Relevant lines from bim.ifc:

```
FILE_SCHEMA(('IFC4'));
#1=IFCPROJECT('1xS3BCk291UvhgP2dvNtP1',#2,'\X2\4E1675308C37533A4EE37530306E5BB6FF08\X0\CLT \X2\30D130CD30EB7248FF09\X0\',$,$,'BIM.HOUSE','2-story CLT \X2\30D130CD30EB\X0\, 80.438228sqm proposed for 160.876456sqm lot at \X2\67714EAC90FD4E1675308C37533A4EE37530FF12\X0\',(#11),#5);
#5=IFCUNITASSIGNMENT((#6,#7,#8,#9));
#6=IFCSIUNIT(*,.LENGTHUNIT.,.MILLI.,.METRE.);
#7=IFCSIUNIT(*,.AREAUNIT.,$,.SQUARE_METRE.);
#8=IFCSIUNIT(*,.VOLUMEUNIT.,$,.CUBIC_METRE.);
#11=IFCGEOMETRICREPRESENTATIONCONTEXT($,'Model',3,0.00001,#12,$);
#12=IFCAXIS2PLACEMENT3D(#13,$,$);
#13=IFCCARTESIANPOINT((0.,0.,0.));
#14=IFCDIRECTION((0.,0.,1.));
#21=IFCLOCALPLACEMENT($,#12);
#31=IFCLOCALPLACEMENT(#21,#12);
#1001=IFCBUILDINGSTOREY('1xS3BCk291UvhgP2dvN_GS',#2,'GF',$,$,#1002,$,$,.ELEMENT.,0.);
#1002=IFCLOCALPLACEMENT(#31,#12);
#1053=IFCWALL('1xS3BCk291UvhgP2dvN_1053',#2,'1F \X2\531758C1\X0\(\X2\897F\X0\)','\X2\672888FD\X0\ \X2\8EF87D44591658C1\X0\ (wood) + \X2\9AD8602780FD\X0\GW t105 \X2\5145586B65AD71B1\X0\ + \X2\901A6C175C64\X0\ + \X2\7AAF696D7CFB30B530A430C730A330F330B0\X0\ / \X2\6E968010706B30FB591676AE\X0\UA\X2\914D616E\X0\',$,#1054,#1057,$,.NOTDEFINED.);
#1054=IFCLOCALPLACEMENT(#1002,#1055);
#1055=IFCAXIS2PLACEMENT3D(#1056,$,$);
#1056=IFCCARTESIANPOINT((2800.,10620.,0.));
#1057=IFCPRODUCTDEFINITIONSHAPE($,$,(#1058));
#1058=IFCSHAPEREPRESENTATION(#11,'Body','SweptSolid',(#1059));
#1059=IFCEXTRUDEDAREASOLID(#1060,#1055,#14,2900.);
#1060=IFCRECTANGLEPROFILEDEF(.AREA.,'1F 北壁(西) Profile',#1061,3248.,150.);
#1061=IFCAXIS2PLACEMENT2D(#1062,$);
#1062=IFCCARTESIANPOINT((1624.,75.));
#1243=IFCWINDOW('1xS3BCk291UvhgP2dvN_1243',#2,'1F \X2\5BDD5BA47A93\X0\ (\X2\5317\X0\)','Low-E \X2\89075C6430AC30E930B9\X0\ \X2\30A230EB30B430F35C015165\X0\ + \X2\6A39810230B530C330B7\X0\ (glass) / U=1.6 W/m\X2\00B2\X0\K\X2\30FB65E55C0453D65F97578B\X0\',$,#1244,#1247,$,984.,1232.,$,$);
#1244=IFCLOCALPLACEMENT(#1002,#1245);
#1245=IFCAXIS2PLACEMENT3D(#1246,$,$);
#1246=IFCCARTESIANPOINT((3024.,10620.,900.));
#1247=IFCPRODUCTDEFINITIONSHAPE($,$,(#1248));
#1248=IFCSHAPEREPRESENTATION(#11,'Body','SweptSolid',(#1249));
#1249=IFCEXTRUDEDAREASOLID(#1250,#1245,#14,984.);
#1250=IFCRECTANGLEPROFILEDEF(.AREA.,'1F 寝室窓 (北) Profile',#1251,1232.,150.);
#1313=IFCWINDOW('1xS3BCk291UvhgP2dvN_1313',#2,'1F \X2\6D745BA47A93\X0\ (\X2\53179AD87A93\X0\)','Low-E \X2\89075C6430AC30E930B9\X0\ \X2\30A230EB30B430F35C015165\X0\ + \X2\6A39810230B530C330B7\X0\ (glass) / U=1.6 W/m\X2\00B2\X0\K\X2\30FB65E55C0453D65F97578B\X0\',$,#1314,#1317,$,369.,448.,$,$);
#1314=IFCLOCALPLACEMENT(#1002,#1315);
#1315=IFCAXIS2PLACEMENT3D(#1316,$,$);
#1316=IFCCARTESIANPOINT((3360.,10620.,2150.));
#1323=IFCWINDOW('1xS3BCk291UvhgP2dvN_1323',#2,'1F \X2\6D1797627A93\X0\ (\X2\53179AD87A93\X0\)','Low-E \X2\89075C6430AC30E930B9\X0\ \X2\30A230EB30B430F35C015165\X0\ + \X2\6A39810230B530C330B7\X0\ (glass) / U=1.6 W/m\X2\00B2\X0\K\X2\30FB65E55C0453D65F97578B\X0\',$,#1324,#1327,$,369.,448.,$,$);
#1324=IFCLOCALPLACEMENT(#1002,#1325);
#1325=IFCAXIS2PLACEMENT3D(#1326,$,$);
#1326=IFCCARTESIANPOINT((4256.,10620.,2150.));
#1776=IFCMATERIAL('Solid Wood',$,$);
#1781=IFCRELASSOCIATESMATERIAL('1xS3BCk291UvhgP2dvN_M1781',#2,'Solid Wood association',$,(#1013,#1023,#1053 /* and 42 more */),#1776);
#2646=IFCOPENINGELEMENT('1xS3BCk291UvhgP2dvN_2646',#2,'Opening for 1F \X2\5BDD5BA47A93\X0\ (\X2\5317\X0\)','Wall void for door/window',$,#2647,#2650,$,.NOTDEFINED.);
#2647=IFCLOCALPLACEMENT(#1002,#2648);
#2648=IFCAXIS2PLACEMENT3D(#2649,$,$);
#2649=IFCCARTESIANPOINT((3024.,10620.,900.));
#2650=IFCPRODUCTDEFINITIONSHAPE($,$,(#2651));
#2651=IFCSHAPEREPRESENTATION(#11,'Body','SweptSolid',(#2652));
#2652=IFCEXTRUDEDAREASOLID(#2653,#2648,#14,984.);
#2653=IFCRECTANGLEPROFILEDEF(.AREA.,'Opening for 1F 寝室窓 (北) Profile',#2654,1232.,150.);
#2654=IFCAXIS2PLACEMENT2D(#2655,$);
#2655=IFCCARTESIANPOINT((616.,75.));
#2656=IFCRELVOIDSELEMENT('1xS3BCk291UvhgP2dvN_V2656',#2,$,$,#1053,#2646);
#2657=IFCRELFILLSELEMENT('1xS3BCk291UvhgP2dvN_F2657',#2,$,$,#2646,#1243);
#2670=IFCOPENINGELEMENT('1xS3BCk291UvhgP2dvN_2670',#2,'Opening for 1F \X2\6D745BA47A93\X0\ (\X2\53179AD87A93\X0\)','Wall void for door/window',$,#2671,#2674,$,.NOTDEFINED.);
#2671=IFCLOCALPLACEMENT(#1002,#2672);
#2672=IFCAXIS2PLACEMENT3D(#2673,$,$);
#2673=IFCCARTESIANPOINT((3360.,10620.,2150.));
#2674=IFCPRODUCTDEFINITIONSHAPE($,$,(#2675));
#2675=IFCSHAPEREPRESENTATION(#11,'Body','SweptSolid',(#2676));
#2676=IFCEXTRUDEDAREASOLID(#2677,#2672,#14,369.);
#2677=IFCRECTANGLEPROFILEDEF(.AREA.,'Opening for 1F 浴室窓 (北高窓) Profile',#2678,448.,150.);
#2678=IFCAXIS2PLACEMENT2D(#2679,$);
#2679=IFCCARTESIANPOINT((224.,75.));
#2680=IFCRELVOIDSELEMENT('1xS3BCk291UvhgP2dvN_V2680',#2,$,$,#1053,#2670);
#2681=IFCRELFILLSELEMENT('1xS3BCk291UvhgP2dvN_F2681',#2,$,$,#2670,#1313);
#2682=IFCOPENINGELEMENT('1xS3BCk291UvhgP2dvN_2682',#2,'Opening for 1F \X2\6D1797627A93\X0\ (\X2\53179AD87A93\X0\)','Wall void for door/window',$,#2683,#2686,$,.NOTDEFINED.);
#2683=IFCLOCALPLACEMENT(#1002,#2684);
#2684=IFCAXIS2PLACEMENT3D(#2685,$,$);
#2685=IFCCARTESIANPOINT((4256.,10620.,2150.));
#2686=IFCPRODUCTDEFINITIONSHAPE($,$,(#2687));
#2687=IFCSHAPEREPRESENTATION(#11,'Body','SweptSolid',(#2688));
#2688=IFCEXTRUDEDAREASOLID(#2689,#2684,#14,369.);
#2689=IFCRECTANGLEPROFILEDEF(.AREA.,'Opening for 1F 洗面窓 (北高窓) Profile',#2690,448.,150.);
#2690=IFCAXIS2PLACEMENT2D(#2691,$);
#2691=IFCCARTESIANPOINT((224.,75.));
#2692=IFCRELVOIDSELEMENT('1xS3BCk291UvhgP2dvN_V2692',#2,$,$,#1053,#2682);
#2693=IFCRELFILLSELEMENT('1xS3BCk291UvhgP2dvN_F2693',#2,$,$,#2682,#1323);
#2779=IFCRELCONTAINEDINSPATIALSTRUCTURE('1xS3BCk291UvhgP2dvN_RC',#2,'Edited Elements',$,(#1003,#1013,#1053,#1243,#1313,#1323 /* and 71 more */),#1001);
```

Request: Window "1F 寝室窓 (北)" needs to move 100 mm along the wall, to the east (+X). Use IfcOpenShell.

```python
import ifcopenshell
import ifcopenshell.api.geometry
import ifcopenshell.util.placement
import ifcopenshell.util.unit

model = ifcopenshell.open("bim.ifc")
unit_scale = ifcopenshell.util.unit.calculate_unit_scale(model)

window = model.by_guid("1xS3BCk291UvhgP2dvN_1243")
opening = window.FillsVoids[0].RelatingOpeningElement
wall = opening.VoidsElements[0].RelatingBuildingElement

wall_matrix = ifcopenshell.util.placement.get_local_placement(wall.ObjectPlacement)
shift = wall_matrix[:3, 0] * 0.1 / unit_scale
before = ifcopenshell.util.placement.get_local_placement(window.ObjectPlacement)[:3, 3].copy()

# The window is not placed relative to its opening, so move both.
for product in (opening, window):
    matrix = ifcopenshell.util.placement.get_local_placement(product.ObjectPlacement)
    matrix[:3, 3] += shift
    ifcopenshell.api.geometry.edit_object_placement(model, product=product, matrix=matrix, is_si=False)

after = ifcopenshell.util.placement.get_local_placement(window.ObjectPlacement)[:3, 3]
print("window moved by", (after - before).round(3) + 0.0)

model.write("bim_v2.ifc")
```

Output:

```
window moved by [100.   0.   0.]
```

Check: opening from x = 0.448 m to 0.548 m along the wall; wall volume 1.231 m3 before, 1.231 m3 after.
